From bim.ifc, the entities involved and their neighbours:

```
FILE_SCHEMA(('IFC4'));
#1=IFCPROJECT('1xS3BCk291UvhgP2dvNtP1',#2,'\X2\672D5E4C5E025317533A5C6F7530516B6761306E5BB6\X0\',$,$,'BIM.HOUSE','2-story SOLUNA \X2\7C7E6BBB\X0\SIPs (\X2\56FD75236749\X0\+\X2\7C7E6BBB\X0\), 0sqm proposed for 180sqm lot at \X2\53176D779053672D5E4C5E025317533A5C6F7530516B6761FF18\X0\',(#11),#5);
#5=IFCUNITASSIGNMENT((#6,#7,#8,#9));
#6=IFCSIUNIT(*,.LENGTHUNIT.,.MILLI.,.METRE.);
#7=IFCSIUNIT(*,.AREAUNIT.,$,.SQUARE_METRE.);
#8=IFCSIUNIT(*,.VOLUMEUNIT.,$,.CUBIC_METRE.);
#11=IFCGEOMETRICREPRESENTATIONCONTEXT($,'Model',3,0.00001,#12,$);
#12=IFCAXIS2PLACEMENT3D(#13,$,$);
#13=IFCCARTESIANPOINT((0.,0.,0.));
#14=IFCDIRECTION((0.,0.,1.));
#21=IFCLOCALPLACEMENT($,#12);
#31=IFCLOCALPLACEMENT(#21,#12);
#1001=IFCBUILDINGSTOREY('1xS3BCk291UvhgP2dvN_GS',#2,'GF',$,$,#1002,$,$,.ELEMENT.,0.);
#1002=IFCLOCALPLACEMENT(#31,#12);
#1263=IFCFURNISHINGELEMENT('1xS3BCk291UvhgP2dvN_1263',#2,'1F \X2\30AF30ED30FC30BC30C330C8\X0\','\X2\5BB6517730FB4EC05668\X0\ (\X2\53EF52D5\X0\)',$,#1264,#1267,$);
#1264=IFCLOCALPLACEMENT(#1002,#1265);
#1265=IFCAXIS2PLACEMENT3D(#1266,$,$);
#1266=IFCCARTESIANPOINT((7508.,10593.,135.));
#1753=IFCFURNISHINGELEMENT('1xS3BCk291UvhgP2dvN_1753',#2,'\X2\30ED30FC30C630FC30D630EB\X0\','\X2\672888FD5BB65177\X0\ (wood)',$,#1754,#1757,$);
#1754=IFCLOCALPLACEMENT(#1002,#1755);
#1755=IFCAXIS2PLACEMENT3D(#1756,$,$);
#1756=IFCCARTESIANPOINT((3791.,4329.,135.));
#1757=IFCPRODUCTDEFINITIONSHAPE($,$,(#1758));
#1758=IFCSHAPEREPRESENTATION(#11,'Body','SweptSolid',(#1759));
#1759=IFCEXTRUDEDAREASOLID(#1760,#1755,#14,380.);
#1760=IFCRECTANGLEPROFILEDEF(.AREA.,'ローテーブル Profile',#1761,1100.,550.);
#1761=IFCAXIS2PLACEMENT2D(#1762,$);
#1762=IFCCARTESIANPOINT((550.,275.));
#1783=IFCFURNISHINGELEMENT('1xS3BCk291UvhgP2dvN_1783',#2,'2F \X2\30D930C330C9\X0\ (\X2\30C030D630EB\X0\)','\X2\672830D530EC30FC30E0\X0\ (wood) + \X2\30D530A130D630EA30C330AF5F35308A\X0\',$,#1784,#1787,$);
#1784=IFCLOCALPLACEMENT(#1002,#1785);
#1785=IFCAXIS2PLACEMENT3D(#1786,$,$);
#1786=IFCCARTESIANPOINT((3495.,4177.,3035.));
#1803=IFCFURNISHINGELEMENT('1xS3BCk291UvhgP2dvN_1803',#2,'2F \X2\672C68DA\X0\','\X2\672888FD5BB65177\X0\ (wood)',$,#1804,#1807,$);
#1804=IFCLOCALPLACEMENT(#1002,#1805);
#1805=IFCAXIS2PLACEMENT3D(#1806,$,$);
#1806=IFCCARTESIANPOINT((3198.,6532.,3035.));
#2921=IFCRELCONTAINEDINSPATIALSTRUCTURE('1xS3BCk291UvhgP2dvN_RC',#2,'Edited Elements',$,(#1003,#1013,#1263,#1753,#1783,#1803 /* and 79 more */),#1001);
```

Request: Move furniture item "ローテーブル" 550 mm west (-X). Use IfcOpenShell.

```python
import ifcopenshell
import ifcopenshell.api.geometry
import ifcopenshell.util.placement

model = ifcopenshell.open("bim.ifc")

item = model.by_id(1753)
matrix = ifcopenshell.util.placement.get_local_placement(item.ObjectPlacement)
matrix[0, 3] -= 550.0
ifcopenshell.api.geometry.edit_object_placement(model, product=item, matrix=matrix, is_si=False)

print(ifcopenshell.util.placement.get_local_placement(item.ObjectPlacement).round(3) + 0.0)

model.write("bim_edited.ifc")
```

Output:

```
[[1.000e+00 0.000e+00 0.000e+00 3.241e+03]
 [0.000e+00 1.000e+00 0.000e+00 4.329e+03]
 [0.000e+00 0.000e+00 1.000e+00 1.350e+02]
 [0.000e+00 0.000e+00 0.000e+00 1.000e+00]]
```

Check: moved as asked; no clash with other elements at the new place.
